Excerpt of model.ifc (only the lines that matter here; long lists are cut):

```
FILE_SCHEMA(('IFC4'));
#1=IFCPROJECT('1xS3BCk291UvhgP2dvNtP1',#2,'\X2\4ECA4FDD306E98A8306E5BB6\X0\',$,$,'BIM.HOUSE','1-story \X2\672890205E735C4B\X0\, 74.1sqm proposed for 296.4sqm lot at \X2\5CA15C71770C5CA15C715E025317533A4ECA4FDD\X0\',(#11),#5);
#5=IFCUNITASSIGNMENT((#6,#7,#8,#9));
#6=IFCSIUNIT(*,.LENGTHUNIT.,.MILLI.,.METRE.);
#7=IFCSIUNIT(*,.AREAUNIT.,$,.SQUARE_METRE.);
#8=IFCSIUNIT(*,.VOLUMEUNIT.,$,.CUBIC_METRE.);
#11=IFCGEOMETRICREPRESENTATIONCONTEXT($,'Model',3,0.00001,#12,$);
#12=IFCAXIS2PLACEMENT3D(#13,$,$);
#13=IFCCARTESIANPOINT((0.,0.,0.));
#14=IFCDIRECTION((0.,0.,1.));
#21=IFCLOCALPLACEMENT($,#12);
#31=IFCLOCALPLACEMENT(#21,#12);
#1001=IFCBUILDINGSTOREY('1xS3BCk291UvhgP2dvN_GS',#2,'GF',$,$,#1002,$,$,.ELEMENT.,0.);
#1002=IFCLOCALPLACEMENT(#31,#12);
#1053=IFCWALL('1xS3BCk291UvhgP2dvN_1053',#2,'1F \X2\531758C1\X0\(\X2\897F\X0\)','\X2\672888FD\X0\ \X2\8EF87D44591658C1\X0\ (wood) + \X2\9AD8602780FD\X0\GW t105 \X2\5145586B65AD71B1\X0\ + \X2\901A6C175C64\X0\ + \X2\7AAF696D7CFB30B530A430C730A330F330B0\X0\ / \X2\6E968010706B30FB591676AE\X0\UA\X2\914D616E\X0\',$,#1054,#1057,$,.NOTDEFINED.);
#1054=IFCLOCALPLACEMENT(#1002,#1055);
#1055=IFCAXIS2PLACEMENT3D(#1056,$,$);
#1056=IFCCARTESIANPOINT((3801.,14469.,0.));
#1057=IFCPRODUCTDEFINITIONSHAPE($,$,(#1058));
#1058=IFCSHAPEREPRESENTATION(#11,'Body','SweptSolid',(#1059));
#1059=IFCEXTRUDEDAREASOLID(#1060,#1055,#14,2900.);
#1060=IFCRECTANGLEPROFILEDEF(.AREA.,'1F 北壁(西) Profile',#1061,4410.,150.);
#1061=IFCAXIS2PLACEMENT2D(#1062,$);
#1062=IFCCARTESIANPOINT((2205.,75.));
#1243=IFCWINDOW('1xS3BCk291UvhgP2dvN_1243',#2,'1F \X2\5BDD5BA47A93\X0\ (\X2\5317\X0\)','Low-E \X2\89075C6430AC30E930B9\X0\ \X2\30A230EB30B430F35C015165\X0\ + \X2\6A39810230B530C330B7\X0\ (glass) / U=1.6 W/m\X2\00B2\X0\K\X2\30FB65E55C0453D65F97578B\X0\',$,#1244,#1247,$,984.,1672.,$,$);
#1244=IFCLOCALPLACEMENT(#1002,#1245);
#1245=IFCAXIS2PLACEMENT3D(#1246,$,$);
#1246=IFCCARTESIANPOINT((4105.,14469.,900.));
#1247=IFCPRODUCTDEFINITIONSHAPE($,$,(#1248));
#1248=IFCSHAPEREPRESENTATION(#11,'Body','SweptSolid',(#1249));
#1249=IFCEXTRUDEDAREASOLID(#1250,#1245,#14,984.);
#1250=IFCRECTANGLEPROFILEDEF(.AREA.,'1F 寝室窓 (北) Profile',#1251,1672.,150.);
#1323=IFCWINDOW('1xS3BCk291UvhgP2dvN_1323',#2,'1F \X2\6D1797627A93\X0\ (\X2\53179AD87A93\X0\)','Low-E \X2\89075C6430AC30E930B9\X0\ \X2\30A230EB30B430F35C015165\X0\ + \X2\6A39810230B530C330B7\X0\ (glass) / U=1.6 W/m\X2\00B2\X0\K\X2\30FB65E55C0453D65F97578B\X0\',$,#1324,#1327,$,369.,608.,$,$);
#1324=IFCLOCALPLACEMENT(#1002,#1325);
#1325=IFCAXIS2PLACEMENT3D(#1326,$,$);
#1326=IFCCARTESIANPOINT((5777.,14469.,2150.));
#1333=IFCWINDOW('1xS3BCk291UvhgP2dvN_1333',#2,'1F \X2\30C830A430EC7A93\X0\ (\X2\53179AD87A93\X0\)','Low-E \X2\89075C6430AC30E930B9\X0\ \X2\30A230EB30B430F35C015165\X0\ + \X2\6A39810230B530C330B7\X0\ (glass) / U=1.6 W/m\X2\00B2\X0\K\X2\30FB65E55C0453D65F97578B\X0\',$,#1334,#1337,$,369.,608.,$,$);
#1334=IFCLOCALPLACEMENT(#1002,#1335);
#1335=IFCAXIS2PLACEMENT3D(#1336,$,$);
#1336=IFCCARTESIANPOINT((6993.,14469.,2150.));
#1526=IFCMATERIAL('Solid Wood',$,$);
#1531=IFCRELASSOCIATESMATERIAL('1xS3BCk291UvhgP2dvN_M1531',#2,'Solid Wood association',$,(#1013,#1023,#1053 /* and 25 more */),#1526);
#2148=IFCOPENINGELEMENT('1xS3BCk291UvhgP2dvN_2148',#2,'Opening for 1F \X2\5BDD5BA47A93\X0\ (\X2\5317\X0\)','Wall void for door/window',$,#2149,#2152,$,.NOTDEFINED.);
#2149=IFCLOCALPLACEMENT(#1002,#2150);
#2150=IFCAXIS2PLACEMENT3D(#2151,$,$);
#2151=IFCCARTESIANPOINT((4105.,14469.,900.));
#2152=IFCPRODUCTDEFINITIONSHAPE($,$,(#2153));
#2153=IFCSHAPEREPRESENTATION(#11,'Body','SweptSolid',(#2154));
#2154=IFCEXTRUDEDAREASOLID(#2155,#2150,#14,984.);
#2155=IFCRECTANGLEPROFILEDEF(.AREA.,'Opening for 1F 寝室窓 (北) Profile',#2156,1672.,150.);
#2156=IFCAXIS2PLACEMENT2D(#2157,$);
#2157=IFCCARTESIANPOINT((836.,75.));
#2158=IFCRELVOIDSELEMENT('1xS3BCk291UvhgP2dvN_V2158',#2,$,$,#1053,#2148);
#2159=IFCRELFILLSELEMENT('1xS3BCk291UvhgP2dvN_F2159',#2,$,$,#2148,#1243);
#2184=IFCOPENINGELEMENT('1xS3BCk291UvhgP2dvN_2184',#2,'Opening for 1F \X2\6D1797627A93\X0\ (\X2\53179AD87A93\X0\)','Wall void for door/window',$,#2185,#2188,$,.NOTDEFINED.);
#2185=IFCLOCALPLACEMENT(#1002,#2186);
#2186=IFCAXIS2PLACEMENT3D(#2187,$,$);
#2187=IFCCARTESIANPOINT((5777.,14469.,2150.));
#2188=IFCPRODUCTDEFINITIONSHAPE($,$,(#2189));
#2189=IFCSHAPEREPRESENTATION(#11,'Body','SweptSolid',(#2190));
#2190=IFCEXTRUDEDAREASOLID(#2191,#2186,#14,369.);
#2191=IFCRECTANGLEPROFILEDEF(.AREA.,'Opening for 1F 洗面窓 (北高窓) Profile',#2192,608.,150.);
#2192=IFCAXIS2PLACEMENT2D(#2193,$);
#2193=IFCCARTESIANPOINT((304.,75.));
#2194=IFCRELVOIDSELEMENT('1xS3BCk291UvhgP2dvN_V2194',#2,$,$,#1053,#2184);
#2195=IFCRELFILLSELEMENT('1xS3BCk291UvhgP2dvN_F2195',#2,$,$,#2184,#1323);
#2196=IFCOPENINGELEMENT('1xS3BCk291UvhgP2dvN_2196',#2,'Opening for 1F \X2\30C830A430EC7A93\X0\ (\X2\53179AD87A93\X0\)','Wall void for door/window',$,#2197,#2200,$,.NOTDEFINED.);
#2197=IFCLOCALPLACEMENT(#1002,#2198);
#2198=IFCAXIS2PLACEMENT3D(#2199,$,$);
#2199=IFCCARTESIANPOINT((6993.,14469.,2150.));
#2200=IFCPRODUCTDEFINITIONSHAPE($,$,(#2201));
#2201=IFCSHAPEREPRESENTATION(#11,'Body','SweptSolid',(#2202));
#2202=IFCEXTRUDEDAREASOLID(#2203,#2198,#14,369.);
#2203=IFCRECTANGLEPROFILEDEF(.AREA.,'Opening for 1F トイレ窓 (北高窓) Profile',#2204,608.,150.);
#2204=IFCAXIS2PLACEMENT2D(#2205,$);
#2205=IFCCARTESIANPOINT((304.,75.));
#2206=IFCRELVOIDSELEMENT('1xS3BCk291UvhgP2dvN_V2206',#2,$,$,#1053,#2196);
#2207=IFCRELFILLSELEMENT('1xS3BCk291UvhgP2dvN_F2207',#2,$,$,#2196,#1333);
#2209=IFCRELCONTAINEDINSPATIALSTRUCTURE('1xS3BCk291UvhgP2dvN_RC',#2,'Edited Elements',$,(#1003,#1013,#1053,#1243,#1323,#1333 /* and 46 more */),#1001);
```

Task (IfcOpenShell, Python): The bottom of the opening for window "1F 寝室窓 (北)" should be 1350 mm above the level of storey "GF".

```python
import numpy as np
import ifcopenshell
import ifcopenshell.api.geometry
import ifcopenshell.geom
import ifcopenshell.util.element
import ifcopenshell.util.placement
import ifcopenshell.util.shape
import ifcopenshell.util.unit

model = ifcopenshell.open("model.ifc")
unit_scale = ifcopenshell.util.unit.calculate_unit_scale(model)

window = model.by_guid("1xS3BCk291UvhgP2dvN_1243")
opening = window.FillsVoids[0].RelatingOpeningElement
storey = ifcopenshell.util.element.get_container(window, ifc_class="IfcBuildingStorey")
level = ifcopenshell.util.placement.get_local_placement(storey.ObjectPlacement)[2, 3]

# The opening's origin need not be at the sill, so measure its lowest point.
shape = ifcopenshell.geom.create_shape(ifcopenshell.geom.settings(), opening)
bottom = ifcopenshell.util.shape.get_shape_bottom_elevation(shape, shape.geometry) / unit_scale
dz = level + 1.35 / unit_scale - bottom

shift = np.array([0.0, 0.0, dz])
# The window is not placed relative to its opening, so move both.
for product in (opening, window):
    matrix = ifcopenshell.util.placement.get_local_placement(product.ObjectPlacement)
    matrix[:3, 3] += shift
    ifcopenshell.api.geometry.edit_object_placement(model, product=product, matrix=matrix, is_si=False)

print(f"moved by {dz * unit_scale:+.3f} m")

model.write("model_edited.ifc")
```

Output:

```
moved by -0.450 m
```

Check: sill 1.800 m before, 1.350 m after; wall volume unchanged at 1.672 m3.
